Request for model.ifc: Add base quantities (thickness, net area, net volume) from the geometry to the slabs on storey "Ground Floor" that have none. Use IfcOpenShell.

First a look at what the model holds.

```python
import ifcopenshell
import ifcopenshell.util.element
import ifcopenshell.util.unit

model = ifcopenshell.open("model.ifc")
print(model.schema)
for unit_type in ("LENGTHUNIT", "AREAUNIT", "VOLUMEUNIT"):
    print(unit_type, ifcopenshell.util.unit.calculate_unit_scale(model, unit_type))
storey = next(s for s in model.by_type("IfcBuildingStorey") if s.Name == "Ground Floor")
slabs = [e for e in ifcopenshell.util.element.get_decomposition(storey) if e.is_a("IfcSlab")]
for e in sorted(slabs, key=lambda e: e.id()):
    print(e.id(), e.is_a(), e.Name, list(ifcopenshell.util.element.get_psets(e, qtos_only=True)), sep=" | ")
```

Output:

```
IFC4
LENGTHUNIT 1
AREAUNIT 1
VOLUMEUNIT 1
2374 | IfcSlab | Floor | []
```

```python
import ifcopenshell
import ifcopenshell.api.pset
import ifcopenshell.geom
import ifcopenshell.util.element
import ifcopenshell.util.shape
import ifcopenshell.util.unit

model = ifcopenshell.open("model.ifc")
unit_scale = ifcopenshell.util.unit.calculate_unit_scale(model)
area_scale = ifcopenshell.util.unit.calculate_unit_scale(model, "AREAUNIT")
volume_scale = ifcopenshell.util.unit.calculate_unit_scale(model, "VOLUMEUNIT")
settings = ifcopenshell.geom.settings()

storey = next(s for s in model.by_type("IfcBuildingStorey") if s.Name == "Ground Floor")
slabs = [e for e in ifcopenshell.util.element.get_decomposition(storey) if e.is_a("IfcSlab")]

for e in sorted(slabs, key=lambda e: e.id()):
    if ifcopenshell.util.element.get_psets(e, qtos_only=True, should_inherit=False):
        continue
    # Geometry comes back in metres, in the element's own axes.
    shape = ifcopenshell.geom.create_shape(settings, e)
    values = {
        "Width": ifcopenshell.util.shape.get_z(shape.geometry) / unit_scale,
        "NetArea": ifcopenshell.util.shape.get_footprint_area(shape.geometry) / area_scale,
        "NetVolume": ifcopenshell.util.shape.get_volume(shape.geometry) / volume_scale,
    }
    qto = ifcopenshell.api.pset.add_qto(model, product=e, name="Qto_SlabBaseQuantities")
    ifcopenshell.api.pset.edit_qto(model, qto=qto, properties=values)
    print(e.id(), {k: round(v, 3) for k, v in values.items()})

model.write("model_v2.ifc")
```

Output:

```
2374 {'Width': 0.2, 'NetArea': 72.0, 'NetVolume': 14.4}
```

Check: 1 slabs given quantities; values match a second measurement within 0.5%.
